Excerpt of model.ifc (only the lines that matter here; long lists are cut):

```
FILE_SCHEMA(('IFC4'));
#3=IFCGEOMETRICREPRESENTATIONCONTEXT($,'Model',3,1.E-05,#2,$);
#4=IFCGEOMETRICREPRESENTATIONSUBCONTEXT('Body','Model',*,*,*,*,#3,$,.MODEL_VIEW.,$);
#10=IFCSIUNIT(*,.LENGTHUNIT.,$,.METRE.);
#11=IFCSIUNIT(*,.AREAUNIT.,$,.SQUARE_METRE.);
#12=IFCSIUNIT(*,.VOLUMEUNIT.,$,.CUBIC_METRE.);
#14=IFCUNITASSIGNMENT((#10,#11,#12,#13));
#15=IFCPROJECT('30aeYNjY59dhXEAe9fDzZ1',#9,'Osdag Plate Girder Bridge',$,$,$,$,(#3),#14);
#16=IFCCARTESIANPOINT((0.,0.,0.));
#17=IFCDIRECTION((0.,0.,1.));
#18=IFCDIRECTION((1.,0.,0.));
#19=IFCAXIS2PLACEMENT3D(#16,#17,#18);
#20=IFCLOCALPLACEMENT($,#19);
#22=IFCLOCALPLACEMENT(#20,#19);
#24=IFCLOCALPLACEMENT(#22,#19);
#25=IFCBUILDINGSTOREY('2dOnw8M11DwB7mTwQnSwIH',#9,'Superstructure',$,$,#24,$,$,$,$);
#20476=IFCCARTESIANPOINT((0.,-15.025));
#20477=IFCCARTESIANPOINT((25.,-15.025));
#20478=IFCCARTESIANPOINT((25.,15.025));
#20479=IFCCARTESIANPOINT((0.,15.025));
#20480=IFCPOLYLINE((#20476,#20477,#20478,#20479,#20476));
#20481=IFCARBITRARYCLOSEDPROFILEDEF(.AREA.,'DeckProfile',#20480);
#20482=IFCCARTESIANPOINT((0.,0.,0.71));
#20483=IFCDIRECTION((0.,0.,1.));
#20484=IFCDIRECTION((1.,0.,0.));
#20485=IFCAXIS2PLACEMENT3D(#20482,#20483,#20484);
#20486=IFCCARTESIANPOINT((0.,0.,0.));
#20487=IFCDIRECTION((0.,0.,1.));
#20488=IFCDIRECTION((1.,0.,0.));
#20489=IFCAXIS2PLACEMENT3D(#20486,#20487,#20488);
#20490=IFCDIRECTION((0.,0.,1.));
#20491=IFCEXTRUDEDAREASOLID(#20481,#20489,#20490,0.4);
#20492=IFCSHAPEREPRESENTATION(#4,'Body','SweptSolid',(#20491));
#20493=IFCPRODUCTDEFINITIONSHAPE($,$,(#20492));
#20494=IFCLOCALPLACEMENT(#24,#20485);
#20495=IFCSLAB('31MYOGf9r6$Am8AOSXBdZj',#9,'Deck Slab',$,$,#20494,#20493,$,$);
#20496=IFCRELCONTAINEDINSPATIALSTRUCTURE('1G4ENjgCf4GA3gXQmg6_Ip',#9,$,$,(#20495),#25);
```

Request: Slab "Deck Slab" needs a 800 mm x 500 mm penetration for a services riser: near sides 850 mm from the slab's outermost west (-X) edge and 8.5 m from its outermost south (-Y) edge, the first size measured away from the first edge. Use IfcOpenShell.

```python
import numpy as np
import ifcopenshell
import ifcopenshell.api.feature
import ifcopenshell.api.geometry
import ifcopenshell.api.root
import ifcopenshell.geom
import ifcopenshell.util.placement
import ifcopenshell.util.representation
import ifcopenshell.util.shape
import ifcopenshell.util.unit

model = ifcopenshell.open("model.ifc")
unit_scale = ifcopenshell.util.unit.calculate_unit_scale(model)
settings = ifcopenshell.geom.settings()


def volume(element):
    """Net volume in cubic metres, openings subtracted."""
    shape = ifcopenshell.geom.create_shape(settings, element)
    return ifcopenshell.util.shape.get_volume(shape.geometry)


slab = model.by_id(20495)
before = volume(slab)

# Extent in the slab's own axes, in metres. The edges named are its -X and -Y sides.
slab_shape = ifcopenshell.geom.create_shape(settings, slab)
vertices = ifcopenshell.util.shape.get_vertices(slab_shape.geometry)
x_min, y_min, bottom = vertices.min(axis=0)
top = vertices[:, 2].max()

opening = ifcopenshell.api.root.create_entity(model, ifc_class="IfcOpeningElement", name="Services riser opening", predefined_type="OPENING")
context = ifcopenshell.util.representation.get_context(model, "Model", "Body", "MODEL_VIEW")
width, depth = 0.8, 0.5
outline = [(0.0, 0.0), (width, 0.0), (width, depth), (0.0, depth), (0.0, 0.0)]
# Overshoot both faces by 50 mm so the cut is clean.
shape = ifcopenshell.api.geometry.add_slab_representation(
    model, context=context, depth=top - bottom + 0.1, polyline=outline
)
ifcopenshell.api.geometry.assign_representation(model, product=opening, representation=shape)

matrix = ifcopenshell.util.placement.get_local_placement(slab.ObjectPlacement)
matrix[:, 3] = matrix @ np.append(np.array([x_min + 0.85, y_min + 8.5, bottom - 0.05]) / unit_scale, 1.0)
ifcopenshell.api.geometry.edit_object_placement(model, product=opening, matrix=matrix, is_si=False)
ifcopenshell.api.feature.add_feature(model, feature=opening, element=slab)

after = volume(slab)

print(f"slab volume {before:.3f} -> {after:.3f} m3")

model.write("model_edited.ifc")
```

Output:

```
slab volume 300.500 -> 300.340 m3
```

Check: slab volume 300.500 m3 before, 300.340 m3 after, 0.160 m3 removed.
